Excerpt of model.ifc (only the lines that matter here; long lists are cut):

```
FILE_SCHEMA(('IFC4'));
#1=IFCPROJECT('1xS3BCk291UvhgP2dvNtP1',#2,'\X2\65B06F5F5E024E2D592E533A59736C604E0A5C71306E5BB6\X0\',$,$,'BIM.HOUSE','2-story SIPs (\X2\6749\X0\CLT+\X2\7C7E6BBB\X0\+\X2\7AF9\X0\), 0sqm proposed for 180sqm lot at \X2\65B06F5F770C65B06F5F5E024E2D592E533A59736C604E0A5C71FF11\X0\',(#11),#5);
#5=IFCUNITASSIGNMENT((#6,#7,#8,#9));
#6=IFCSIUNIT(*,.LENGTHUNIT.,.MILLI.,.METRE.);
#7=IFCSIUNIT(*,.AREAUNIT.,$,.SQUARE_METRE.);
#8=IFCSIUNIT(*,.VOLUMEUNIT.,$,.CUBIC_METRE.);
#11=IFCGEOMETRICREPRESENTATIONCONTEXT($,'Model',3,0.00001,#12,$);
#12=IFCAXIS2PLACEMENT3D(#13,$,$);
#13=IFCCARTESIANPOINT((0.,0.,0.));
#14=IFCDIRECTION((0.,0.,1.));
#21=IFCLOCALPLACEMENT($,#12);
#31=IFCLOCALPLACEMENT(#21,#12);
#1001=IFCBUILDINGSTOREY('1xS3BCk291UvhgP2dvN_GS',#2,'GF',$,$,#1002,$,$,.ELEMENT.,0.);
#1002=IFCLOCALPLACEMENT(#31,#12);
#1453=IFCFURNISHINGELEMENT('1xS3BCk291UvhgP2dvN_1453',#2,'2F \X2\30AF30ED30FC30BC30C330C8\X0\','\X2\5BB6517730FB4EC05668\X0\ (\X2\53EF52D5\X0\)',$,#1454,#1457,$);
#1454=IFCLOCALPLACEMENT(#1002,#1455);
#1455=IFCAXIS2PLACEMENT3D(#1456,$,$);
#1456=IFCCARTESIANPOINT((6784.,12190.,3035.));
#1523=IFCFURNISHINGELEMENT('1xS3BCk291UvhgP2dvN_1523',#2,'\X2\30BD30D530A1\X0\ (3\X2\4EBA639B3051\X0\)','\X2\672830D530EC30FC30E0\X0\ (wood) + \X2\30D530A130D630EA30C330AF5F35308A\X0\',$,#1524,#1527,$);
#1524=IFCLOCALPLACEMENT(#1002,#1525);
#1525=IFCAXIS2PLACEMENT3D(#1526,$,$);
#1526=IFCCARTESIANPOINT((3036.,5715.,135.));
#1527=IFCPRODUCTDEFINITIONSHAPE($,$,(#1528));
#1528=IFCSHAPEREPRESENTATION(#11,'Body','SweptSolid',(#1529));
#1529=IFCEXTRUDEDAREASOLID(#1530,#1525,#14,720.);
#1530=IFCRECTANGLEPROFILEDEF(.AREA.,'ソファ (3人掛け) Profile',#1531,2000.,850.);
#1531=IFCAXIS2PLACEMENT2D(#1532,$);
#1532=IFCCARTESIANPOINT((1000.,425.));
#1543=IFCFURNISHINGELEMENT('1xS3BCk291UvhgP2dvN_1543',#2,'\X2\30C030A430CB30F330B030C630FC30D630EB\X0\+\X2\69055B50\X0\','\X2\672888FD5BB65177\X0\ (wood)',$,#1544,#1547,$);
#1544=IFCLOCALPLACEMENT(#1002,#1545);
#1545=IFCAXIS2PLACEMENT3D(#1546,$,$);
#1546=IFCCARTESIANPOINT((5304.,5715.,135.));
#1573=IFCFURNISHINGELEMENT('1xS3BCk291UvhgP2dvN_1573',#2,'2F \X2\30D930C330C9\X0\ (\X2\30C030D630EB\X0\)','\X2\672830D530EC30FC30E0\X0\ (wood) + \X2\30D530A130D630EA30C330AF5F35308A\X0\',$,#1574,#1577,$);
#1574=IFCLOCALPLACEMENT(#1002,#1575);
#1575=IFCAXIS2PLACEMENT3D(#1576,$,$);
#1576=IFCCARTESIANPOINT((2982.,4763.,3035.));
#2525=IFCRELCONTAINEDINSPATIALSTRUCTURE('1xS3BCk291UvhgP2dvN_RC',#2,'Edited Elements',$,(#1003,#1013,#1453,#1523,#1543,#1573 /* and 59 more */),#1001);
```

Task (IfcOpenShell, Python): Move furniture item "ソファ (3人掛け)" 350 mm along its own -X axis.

```python
import ifcopenshell
import ifcopenshell.api.geometry
import ifcopenshell.util.placement
import ifcopenshell.util.unit

model = ifcopenshell.open("model.ifc")
unit_scale = ifcopenshell.util.unit.calculate_unit_scale(model)

item = model.by_guid("1xS3BCk291UvhgP2dvN_1523")
matrix = ifcopenshell.util.placement.get_local_placement(item.ObjectPlacement)
matrix[:3, 3] -= matrix[:3, 0] * 0.35 / unit_scale
ifcopenshell.api.geometry.edit_object_placement(model, product=item, matrix=matrix, is_si=False)

print(ifcopenshell.util.placement.get_local_placement(item.ObjectPlacement).round(3) + 0.0)

model.write("model_rev.ifc")
```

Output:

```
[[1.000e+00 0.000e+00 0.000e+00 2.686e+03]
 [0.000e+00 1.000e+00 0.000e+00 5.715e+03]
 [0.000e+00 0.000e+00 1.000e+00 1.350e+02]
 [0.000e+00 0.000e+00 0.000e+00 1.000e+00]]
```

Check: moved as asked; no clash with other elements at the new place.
